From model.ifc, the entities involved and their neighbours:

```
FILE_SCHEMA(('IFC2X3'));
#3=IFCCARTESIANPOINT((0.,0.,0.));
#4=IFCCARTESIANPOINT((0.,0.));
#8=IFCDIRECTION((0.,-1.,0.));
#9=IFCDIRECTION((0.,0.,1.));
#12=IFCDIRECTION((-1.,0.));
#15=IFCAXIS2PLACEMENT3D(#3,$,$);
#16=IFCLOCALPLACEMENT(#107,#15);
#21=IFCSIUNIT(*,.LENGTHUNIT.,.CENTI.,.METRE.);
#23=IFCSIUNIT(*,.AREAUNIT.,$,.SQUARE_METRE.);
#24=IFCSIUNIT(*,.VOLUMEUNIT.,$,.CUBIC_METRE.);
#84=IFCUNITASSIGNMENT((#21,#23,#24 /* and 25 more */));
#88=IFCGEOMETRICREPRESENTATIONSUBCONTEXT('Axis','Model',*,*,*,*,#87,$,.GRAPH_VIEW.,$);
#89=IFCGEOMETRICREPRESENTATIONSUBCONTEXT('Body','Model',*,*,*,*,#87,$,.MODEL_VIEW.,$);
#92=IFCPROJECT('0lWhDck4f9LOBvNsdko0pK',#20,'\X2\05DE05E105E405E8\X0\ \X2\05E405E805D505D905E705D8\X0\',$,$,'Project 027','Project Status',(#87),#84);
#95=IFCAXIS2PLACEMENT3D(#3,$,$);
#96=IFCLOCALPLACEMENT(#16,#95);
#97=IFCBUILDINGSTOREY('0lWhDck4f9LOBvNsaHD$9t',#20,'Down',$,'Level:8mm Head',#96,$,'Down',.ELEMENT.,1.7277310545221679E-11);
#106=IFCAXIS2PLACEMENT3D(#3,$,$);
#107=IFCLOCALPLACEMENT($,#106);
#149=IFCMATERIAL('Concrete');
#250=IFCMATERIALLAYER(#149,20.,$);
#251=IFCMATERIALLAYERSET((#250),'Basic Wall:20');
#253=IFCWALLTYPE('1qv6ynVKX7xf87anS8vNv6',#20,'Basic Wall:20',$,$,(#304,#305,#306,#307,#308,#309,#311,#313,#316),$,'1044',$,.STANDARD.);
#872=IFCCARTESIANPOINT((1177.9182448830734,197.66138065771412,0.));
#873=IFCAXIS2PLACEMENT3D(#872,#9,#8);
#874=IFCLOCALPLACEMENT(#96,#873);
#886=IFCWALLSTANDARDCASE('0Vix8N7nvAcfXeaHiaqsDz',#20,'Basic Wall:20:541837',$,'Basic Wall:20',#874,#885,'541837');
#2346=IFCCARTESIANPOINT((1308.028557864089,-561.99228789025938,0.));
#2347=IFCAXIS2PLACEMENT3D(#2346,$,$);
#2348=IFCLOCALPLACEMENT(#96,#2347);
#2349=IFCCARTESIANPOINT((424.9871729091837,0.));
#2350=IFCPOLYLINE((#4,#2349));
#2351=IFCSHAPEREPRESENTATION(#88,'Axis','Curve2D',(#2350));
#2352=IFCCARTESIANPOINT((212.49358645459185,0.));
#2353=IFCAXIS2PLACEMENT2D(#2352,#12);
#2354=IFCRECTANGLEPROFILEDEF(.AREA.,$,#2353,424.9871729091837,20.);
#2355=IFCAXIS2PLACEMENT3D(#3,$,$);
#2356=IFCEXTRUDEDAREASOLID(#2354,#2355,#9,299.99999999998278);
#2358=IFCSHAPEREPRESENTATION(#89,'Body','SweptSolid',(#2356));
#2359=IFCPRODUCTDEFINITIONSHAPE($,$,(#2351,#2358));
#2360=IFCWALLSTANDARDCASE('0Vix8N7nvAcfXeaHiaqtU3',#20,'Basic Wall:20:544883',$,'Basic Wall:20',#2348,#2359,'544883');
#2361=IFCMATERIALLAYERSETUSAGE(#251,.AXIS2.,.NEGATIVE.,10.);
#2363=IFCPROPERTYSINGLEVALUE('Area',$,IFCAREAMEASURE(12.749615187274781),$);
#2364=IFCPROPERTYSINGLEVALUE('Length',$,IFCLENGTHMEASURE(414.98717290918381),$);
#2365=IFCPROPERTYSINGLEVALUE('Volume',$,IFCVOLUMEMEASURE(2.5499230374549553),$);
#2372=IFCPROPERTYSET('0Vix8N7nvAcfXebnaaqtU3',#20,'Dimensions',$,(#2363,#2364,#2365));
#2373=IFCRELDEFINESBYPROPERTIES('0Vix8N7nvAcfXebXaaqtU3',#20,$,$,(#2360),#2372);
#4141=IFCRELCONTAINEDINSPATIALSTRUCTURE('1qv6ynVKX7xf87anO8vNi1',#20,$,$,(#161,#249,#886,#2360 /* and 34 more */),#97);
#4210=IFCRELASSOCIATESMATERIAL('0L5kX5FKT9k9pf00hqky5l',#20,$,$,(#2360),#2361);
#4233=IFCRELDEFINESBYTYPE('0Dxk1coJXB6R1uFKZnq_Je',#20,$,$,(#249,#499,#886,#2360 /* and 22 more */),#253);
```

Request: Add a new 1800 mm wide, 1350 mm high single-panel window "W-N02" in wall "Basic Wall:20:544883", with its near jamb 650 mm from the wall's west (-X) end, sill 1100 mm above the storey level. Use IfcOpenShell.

```python
import numpy as np
import ifcopenshell
import ifcopenshell.api.feature
import ifcopenshell.api.geometry
import ifcopenshell.api.pset
import ifcopenshell.api.root
import ifcopenshell.api.spatial
import ifcopenshell.api.type
import ifcopenshell.geom
import ifcopenshell.util.element
import ifcopenshell.util.placement
import ifcopenshell.util.representation
import ifcopenshell.util.shape
import ifcopenshell.util.unit

model = ifcopenshell.open("model.ifc")
unit_scale = ifcopenshell.util.unit.calculate_unit_scale(model)
area_scale = ifcopenshell.util.unit.calculate_unit_scale(model, "AREAUNIT")
volume_scale = ifcopenshell.util.unit.calculate_unit_scale(model, "VOLUMEUNIT")
settings = ifcopenshell.geom.settings()


def volume(element):
    """Net volume in cubic metres, openings subtracted."""
    shape = ifcopenshell.geom.create_shape(settings, element)
    return ifcopenshell.util.shape.get_volume(shape.geometry)


wall = model.by_id(2360)
storey = ifcopenshell.util.element.get_container(wall, ifc_class="IfcBuildingStorey")
context = ifcopenshell.util.representation.get_context(model, "Model", "Body", "MODEL_VIEW")
before = volume(wall)

width, height, from_end, sill = 1.8, 1.35, 0.65, 1.1  # metres

# The wall runs along its own X axis, and the end named is its -X end.
wall_shape = ifcopenshell.geom.create_shape(settings, wall)
x, y, z = ifcopenshell.util.shape.get_vertices(wall_shape.geometry).T
start = x.min() + from_end
face, thickness = float(y.min()), float(y.max() - y.min())
wall_matrix = ifcopenshell.util.placement.get_local_placement(wall.ObjectPlacement)
level = ifcopenshell.util.placement.get_local_placement(storey.ObjectPlacement)[2, 3]


def in_wall(x, y):
    """Placement at x, y metres in the wall's axes, at sill height."""
    matrix = wall_matrix.copy()
    matrix[:, 3] = wall_matrix @ np.array([x / unit_scale, y / unit_scale, 0.0, 1.0])
    matrix[2, 3] = level + sill / unit_scale
    return matrix


# Opening: a box that overshoots both wall faces by 50 mm.
opening = ifcopenshell.api.root.create_entity(model, ifc_class="IfcOpeningElement")
box = ifcopenshell.api.geometry.add_wall_representation(
    model, context=context, length=width, height=height, thickness=thickness + 0.1
)
ifcopenshell.api.geometry.assign_representation(model, product=opening, representation=box)
ifcopenshell.api.geometry.edit_object_placement(model, product=opening, matrix=in_wall(start, face - 0.05), is_si=False)
ifcopenshell.api.feature.add_feature(model, feature=opening, element=wall)

window = ifcopenshell.api.root.create_entity(model, ifc_class="IfcWindow", name="W-N02")
window.OverallWidth, window.OverallHeight = width / unit_scale, height / unit_scale
body = ifcopenshell.api.geometry.add_window_representation(
    model,
    context=context,
    overall_width=window.OverallWidth,
    overall_height=window.OverallHeight,
    partition_type="SINGLE_PANEL",
)
ifcopenshell.api.geometry.assign_representation(model, product=window, representation=body)
ifcopenshell.api.spatial.assign_container(model, products=[window], relating_structure=storey)
fills = ifcopenshell.api.feature.add_filling(model, opening=opening, element=window)
fills.OwnerHistory = window.OwnerHistory  # required in IFC2X3

# IFC2X3 keeps the operation on the window style.
style = ifcopenshell.api.root.create_entity(model, ifc_class="IfcWindowStyle", name="W-N02")
style.OperationType, style.ConstructionType = "SINGLE_PANEL", "NOTDEFINED"
style.ParameterTakesPrecedence = style.Sizeable = False
ifcopenshell.api.type.assign_type(model, related_objects=[window], relating_type=style)

# Centre the window in the wall's thickness.
ifcopenshell.api.geometry.edit_object_placement(model, product=window, matrix=in_wall(start, face), is_si=False)
window_shape = ifcopenshell.geom.create_shape(settings, window)
depth = ifcopenshell.util.shape.get_vertices(window_shape.geometry)[:, 1]
offset = face + thickness / 2 - (depth.min() + depth.max()) / 2
ifcopenshell.api.geometry.edit_object_placement(model, product=window, matrix=in_wall(start, offset), is_si=False)

after = volume(wall)

# Update the wall's stored quantities.
pset = model.by_id(ifcopenshell.util.element.get_pset(wall, "Dimensions", should_inherit=False)["id"])
ifcopenshell.api.pset.edit_pset(model, pset=pset, properties={
    "Area": model.create_entity("IfcAreaMeasure", after / thickness / area_scale),
    "Volume": model.create_entity("IfcVolumeMeasure", after / volume_scale),
})

print(f"wall volume {before:.3f} -> {after:.3f} m3")

model.write("model-out.ifc")
```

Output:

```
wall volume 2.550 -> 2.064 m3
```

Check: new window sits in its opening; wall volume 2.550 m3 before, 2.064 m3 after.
